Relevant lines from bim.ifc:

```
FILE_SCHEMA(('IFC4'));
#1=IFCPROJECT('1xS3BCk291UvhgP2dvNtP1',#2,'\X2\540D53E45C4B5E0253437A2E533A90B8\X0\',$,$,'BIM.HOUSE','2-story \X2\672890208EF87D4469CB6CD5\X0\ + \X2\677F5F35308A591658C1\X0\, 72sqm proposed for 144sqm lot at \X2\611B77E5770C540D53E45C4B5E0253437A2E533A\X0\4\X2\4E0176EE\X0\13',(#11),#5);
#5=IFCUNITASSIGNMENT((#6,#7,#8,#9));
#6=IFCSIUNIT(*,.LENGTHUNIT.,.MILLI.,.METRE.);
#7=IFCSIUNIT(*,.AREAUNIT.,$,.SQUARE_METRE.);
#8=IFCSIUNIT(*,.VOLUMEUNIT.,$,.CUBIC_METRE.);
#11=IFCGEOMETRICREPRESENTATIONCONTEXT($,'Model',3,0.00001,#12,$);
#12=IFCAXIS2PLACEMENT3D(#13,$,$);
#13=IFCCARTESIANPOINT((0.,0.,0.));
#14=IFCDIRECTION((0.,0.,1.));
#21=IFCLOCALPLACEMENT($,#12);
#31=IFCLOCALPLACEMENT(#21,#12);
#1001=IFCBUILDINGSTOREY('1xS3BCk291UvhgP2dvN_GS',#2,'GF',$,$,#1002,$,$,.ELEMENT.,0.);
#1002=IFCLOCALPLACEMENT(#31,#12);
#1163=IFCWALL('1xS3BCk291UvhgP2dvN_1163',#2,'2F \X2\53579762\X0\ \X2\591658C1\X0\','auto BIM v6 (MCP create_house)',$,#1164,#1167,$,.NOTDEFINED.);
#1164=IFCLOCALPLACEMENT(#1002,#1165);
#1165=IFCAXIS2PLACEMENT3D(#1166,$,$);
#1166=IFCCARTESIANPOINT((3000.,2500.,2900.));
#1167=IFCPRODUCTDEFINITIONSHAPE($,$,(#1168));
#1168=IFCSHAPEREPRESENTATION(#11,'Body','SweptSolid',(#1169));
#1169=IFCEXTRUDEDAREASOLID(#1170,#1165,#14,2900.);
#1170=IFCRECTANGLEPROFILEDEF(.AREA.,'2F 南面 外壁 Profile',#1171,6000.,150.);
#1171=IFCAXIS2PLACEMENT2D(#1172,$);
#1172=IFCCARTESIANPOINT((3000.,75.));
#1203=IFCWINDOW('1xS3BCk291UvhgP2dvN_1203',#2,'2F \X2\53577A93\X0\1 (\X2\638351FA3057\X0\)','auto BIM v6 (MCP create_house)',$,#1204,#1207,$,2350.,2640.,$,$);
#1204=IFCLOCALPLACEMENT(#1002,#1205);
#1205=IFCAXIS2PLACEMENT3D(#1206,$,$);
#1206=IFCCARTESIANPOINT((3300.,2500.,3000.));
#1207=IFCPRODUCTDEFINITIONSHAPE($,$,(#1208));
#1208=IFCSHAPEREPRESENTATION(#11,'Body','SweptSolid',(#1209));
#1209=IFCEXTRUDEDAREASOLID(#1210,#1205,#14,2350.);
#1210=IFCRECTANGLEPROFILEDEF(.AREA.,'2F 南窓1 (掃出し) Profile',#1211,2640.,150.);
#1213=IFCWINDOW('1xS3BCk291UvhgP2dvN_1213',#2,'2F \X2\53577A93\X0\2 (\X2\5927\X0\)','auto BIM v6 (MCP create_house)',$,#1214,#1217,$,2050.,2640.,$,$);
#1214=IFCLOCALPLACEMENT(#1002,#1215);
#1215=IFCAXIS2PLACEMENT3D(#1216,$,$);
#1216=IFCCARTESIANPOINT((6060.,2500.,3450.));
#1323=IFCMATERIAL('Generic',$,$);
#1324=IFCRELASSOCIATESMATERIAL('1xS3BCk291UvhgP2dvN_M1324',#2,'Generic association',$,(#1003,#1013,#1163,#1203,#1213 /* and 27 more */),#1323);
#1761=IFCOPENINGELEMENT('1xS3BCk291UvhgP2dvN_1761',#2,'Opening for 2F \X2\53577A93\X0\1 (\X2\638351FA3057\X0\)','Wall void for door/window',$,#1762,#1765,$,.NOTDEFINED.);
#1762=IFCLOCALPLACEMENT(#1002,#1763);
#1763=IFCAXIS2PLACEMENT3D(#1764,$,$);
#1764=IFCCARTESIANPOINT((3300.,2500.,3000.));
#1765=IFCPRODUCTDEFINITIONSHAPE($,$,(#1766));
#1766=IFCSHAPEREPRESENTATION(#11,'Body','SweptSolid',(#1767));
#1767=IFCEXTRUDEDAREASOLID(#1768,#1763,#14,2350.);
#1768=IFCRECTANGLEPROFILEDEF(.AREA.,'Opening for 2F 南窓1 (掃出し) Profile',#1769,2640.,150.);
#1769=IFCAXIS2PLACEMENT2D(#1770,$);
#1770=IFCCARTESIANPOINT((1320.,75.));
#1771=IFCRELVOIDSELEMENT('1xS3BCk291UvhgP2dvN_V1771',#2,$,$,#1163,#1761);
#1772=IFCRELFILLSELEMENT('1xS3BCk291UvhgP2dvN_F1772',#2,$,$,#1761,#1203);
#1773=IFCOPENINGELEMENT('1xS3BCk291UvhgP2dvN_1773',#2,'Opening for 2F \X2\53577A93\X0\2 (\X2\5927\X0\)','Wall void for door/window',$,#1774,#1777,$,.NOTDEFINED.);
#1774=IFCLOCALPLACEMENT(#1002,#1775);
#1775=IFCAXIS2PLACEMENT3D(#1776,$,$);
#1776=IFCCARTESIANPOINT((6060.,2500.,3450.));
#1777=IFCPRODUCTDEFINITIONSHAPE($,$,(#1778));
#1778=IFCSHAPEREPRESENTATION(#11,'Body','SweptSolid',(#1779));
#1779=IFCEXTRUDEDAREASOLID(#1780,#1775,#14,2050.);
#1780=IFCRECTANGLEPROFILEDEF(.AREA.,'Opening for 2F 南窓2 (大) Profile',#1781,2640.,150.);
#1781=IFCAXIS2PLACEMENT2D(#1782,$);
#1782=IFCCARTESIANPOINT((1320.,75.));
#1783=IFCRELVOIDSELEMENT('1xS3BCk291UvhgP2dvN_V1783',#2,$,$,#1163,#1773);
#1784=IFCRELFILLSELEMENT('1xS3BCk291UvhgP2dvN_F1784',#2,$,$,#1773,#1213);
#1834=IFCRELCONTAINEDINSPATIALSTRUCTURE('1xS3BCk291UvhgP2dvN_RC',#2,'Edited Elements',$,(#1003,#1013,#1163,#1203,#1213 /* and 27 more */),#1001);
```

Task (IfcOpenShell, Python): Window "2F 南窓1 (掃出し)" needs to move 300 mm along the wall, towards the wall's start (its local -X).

```python
import ifcopenshell
import ifcopenshell.api.geometry
import ifcopenshell.util.placement

model = ifcopenshell.open("bim.ifc")

window = model.by_id(1203)
opening = window.FillsVoids[0].RelatingOpeningElement
wall = opening.VoidsElements[0].RelatingBuildingElement

wall_matrix = ifcopenshell.util.placement.get_local_placement(wall.ObjectPlacement)
shift = wall_matrix[:3, 0] * -300.0
before = ifcopenshell.util.placement.get_local_placement(window.ObjectPlacement)[:3, 3].copy()

# The window is not placed relative to its opening, so move both.
for product in (opening, window):
    matrix = ifcopenshell.util.placement.get_local_placement(product.ObjectPlacement)
    matrix[:3, 3] += shift
    ifcopenshell.api.geometry.edit_object_placement(model, product=product, matrix=matrix, is_si=False)

after = ifcopenshell.util.placement.get_local_placement(window.ObjectPlacement)[:3, 3]
print("window moved by", (after - before).round(3) + 0.0)

model.write("bim_v2.ifc")
```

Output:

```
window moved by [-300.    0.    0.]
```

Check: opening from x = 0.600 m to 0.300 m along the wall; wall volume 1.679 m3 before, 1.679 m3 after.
